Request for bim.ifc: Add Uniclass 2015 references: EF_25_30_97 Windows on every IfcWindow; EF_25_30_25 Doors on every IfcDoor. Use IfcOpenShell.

First a look at what the model holds.

```python
import ifcopenshell

model = ifcopenshell.open("bim.ifc")
print(model.schema)
print("classifications:", [c.Name for c in model.by_type("IfcClassification")])
for ifc_class in ("IfcDoor", "IfcRoof", "IfcStair", "IfcWall", "IfcWindow"):
    print(ifc_class, len(model.by_type(ifc_class)))
```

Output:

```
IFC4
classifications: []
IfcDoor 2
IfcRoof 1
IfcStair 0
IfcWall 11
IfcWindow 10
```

```python
import ifcopenshell
import ifcopenshell.api.classification

model = ifcopenshell.open("bim.ifc")

system = ifcopenshell.api.classification.add_classification(model, classification="Uniclass 2015")

codes = {
    "IfcWindow": ("EF_25_30_97", "Windows"),
    "IfcDoor": ("EF_25_30_25", "Doors"),
}
for ifc_class, (code, name) in codes.items():
    products = model.by_type(ifc_class)
    ifcopenshell.api.classification.add_reference(
        model, products=products, classification=system, identification=code, name=name
    )
    print(code, len(products))

model.write("bim_edited.ifc")
```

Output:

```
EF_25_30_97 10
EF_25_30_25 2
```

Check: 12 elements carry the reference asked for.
